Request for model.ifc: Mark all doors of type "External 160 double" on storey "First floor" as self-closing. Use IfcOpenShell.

First a look at what the model holds.

```python
import ifcopenshell
import ifcopenshell.util.element

model = ifcopenshell.open("model.ifc")
print(model.schema)
storey = next(s for s in model.by_type("IfcBuildingStorey") if s.Name == "First floor")
doors = [e for e in ifcopenshell.util.element.get_decomposition(storey) if e.is_a("IfcDoor")]
seen = {}
for e in doors:
    element_type = ifcopenshell.util.element.get_type(e)
    key = (element_type.Name if element_type != e and element_type else None, ifcopenshell.util.element.get_pset(e, "Pset_DoorCommon", "SelfClosing"))
    seen[key] = seen.get(key, 0) + 1
for (name, value), count in sorted(seen.items(), key=str):
    print(count, "x", name, "|", value)
```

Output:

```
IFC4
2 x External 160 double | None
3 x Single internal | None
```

```python
import ifcopenshell
import ifcopenshell.api.pset
import ifcopenshell.util.element

model = ifcopenshell.open("model.ifc")

storey = next(s for s in model.by_type("IfcBuildingStorey") if s.Name == "First floor")
doors = [e for e in ifcopenshell.util.element.get_decomposition(storey) if e.is_a("IfcDoor")]

count = 0
for e in doors:
    element_type = ifcopenshell.util.element.get_type(e)
    if element_type in (None, e) or element_type.Name != "External 160 double":
        continue
    # add_pset returns the element's existing set when there is one.
    pset = ifcopenshell.api.pset.add_pset(model, product=e, name="Pset_DoorCommon")
    ifcopenshell.api.pset.edit_pset(model, pset=pset, properties={"SelfClosing": True})
    count += 1

print(count, "doors updated")

model.write("model-out.ifc")
```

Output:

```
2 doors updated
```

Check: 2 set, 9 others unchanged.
